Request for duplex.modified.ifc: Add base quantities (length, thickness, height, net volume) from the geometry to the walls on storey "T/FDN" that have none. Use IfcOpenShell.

First a look at what the model holds.

```python
import ifcopenshell
import ifcopenshell.util.element
import ifcopenshell.util.unit

model = ifcopenshell.open("duplex.modified.ifc")
print(model.schema)
for unit_type in ("LENGTHUNIT", "AREAUNIT", "VOLUMEUNIT"):
    print(unit_type, ifcopenshell.util.unit.calculate_unit_scale(model, unit_type))
storey = next(s for s in model.by_type("IfcBuildingStorey") if s.Name == "T/FDN")
walls = [e for e in ifcopenshell.util.element.get_decomposition(storey) if e.is_a("IfcWall")]
for e in sorted(walls, key=lambda e: e.id()):
    print(e.id(), e.is_a(), e.Name, list(ifcopenshell.util.element.get_psets(e, qtos_only=True)), sep=" | ")
```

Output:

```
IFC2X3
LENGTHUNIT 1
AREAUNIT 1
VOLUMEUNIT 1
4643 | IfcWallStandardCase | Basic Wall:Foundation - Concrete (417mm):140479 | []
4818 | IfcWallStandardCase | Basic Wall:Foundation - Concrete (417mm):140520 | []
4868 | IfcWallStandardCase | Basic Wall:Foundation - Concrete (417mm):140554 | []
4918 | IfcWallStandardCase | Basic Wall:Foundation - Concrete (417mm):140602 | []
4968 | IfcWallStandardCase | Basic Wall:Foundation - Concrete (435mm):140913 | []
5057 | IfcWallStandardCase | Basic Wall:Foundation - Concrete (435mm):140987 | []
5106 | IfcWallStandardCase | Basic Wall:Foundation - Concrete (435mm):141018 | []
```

```python
import ifcopenshell
import ifcopenshell.api.pset
import ifcopenshell.geom
import ifcopenshell.util.element
import ifcopenshell.util.shape
import ifcopenshell.util.unit

model = ifcopenshell.open("duplex.modified.ifc")
unit_scale = ifcopenshell.util.unit.calculate_unit_scale(model)
volume_scale = ifcopenshell.util.unit.calculate_unit_scale(model, "VOLUMEUNIT")
settings = ifcopenshell.geom.settings()

storey = next(s for s in model.by_type("IfcBuildingStorey") if s.Name == "T/FDN")
walls = [e for e in ifcopenshell.util.element.get_decomposition(storey) if e.is_a("IfcWall")]

for e in sorted(walls, key=lambda e: e.id()):
    if ifcopenshell.util.element.get_psets(e, qtos_only=True, should_inherit=False):
        continue
    # Geometry comes back in metres, in the element's own axes.
    shape = ifcopenshell.geom.create_shape(settings, e)
    values = {
        "Length": ifcopenshell.util.shape.get_x(shape.geometry) / unit_scale,
        "Width": ifcopenshell.util.shape.get_y(shape.geometry) / unit_scale,
        "Height": ifcopenshell.util.shape.get_z(shape.geometry) / unit_scale,
        "NetVolume": ifcopenshell.util.shape.get_volume(shape.geometry) / volume_scale,
    }
    qto = ifcopenshell.api.pset.add_qto(model, product=e, name="BaseQuantities")
    ifcopenshell.api.pset.edit_qto(model, qto=qto, properties=values)
    print(e.id(), {k: round(v, 3) for k, v in values.items()})

model.write("duplex.modified_v2.ifc")
```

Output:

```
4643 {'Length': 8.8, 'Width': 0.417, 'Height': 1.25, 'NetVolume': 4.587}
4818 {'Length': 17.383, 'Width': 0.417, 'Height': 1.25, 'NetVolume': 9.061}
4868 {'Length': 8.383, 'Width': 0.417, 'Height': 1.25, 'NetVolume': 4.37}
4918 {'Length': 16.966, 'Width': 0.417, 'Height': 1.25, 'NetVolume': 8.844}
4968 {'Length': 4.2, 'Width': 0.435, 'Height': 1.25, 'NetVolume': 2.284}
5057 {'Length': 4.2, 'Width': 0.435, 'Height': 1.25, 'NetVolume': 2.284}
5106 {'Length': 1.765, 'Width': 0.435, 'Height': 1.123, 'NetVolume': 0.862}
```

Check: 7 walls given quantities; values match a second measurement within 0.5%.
